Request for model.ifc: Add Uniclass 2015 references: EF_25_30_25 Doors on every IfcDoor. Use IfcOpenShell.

First a look at what the model holds.

```python
import ifcopenshell

model = ifcopenshell.open("model.ifc")
print(model.schema)
print("classifications:", [c.Name for c in model.by_type("IfcClassification")])
for ifc_class in ("IfcDoor", "IfcRoof", "IfcStair", "IfcWall", "IfcWindow"):
    print(ifc_class, len(model.by_type(ifc_class)))
```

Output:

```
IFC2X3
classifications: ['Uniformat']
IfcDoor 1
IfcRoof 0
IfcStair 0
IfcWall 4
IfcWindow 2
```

```python
import ifcopenshell
import ifcopenshell.api.classification

model = ifcopenshell.open("model.ifc")

# IFC2X3 requires Source and Edition and has no link from the project to the system.
system = model.create_entity("IfcClassification", Source="NBS", Edition="2015", Name="Uniclass 2015")

codes = {
    "IfcDoor": ("EF_25_30_25", "Doors"),
}
for ifc_class, (code, name) in codes.items():
    products = model.by_type(ifc_class)
    ifcopenshell.api.classification.add_reference(
        model, products=products, classification=system, identification=code, name=name
    )
    print(code, len(products))

model.write("model-out.ifc")
```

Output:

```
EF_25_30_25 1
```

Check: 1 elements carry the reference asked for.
